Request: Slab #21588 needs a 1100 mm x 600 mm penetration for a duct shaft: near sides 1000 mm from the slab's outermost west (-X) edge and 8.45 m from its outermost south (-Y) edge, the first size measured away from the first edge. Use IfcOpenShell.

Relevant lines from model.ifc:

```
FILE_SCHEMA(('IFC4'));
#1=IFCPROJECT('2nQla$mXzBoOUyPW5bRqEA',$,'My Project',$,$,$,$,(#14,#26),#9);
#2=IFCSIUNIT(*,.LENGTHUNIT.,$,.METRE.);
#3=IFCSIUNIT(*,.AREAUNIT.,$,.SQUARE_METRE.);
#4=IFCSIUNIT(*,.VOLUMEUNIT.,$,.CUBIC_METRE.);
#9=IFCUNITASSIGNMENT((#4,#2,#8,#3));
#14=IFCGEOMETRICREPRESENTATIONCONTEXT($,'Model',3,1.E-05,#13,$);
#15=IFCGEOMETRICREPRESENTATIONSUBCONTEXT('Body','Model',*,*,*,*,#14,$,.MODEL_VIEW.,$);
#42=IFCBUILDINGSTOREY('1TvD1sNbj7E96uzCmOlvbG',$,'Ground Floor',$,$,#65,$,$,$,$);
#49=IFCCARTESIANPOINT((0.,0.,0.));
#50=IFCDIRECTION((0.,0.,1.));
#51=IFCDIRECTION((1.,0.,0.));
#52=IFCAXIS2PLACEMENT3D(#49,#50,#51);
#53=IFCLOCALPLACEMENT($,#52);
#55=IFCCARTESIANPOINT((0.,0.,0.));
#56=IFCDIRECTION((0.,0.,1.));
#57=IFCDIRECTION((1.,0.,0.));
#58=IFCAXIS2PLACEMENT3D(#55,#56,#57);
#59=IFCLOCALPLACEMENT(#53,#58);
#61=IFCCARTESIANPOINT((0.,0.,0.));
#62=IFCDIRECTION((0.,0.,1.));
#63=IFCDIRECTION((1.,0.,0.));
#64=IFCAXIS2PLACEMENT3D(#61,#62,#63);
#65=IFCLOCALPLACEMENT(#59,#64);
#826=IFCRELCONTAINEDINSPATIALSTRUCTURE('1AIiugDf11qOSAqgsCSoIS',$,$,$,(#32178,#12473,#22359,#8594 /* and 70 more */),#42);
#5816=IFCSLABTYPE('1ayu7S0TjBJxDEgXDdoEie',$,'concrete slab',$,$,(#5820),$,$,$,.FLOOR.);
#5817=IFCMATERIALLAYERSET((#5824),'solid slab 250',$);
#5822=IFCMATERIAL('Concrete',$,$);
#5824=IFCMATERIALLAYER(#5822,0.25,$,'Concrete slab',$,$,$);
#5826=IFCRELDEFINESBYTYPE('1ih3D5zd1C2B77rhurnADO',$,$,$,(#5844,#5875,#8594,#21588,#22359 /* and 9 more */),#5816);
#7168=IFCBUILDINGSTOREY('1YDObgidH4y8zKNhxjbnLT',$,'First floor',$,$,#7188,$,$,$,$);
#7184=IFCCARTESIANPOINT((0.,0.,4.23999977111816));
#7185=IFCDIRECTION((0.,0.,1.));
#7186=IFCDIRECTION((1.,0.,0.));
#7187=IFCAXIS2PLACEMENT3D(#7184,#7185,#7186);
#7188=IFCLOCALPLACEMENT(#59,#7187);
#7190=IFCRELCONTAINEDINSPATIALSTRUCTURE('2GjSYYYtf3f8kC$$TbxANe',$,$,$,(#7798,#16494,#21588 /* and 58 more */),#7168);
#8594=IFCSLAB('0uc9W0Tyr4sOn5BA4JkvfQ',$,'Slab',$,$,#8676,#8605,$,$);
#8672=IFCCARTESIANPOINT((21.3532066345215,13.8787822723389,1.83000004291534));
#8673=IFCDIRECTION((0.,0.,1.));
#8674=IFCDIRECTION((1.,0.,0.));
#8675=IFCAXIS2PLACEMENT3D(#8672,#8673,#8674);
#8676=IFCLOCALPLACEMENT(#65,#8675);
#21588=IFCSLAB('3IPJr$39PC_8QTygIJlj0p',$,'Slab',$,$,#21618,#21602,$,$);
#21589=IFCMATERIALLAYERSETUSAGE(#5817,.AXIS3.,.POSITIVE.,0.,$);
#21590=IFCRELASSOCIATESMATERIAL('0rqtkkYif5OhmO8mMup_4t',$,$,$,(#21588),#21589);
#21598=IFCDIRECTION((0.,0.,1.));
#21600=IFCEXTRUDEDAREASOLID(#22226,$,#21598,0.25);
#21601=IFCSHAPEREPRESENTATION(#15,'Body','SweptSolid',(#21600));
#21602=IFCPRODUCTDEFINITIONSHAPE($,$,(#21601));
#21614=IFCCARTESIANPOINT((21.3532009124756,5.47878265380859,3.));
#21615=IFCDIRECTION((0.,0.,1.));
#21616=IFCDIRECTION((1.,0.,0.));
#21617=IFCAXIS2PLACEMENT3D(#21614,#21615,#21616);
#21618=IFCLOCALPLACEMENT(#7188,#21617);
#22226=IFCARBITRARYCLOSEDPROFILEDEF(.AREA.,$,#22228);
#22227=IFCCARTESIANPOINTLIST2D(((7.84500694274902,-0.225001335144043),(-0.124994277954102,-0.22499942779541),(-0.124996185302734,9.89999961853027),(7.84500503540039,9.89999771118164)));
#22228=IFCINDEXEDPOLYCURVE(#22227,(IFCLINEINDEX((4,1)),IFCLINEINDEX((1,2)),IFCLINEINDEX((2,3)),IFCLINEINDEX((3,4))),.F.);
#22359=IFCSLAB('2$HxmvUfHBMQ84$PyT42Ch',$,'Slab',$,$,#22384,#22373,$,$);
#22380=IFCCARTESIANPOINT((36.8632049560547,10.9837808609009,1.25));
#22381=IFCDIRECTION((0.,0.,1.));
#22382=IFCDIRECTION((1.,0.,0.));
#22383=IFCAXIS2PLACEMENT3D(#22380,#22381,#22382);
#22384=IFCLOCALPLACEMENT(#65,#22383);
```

```python
import numpy as np
import ifcopenshell
import ifcopenshell.api.feature
import ifcopenshell.api.geometry
import ifcopenshell.api.root
import ifcopenshell.geom
import ifcopenshell.util.placement
import ifcopenshell.util.representation
import ifcopenshell.util.shape
import ifcopenshell.util.unit

model = ifcopenshell.open("model.ifc")
unit_scale = ifcopenshell.util.unit.calculate_unit_scale(model)
settings = ifcopenshell.geom.settings()


def volume(element):
    """Net volume in cubic metres, openings subtracted."""
    shape = ifcopenshell.geom.create_shape(settings, element)
    return ifcopenshell.util.shape.get_volume(shape.geometry)


slab = model.by_guid("3IPJr$39PC_8QTygIJlj0p")
before = volume(slab)

# Extent in the slab's own axes, in metres. The edges named are its -X and -Y sides.
slab_shape = ifcopenshell.geom.create_shape(settings, slab)
vertices = ifcopenshell.util.shape.get_vertices(slab_shape.geometry)
x_min, y_min, bottom = vertices.min(axis=0)
top = vertices[:, 2].max()

opening = ifcopenshell.api.root.create_entity(model, ifc_class="IfcOpeningElement", name="Duct shaft opening", predefined_type="OPENING")
context = ifcopenshell.util.representation.get_context(model, "Model", "Body", "MODEL_VIEW")
width, depth = 1.1, 0.6
outline = [(0.0, 0.0), (width, 0.0), (width, depth), (0.0, depth), (0.0, 0.0)]
# Overshoot both faces by 50 mm so the cut is clean.
shape = ifcopenshell.api.geometry.add_slab_representation(
    model, context=context, depth=top - bottom + 0.1, polyline=outline
)
ifcopenshell.api.geometry.assign_representation(model, product=opening, representation=shape)

matrix = ifcopenshell.util.placement.get_local_placement(slab.ObjectPlacement)
matrix[:, 3] = matrix @ np.append(np.array([x_min + 1, y_min + 8.45, bottom - 0.05]) / unit_scale, 1.0)
ifcopenshell.api.geometry.edit_object_placement(model, product=opening, matrix=matrix, is_si=False)
ifcopenshell.api.feature.add_feature(model, feature=opening, element=slab)

after = volume(slab)

print(f"slab volume {before:.3f} -> {after:.3f} m3")

model.write("model-out.ifc")
```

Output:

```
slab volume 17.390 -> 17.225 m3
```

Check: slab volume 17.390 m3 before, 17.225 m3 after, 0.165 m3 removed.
